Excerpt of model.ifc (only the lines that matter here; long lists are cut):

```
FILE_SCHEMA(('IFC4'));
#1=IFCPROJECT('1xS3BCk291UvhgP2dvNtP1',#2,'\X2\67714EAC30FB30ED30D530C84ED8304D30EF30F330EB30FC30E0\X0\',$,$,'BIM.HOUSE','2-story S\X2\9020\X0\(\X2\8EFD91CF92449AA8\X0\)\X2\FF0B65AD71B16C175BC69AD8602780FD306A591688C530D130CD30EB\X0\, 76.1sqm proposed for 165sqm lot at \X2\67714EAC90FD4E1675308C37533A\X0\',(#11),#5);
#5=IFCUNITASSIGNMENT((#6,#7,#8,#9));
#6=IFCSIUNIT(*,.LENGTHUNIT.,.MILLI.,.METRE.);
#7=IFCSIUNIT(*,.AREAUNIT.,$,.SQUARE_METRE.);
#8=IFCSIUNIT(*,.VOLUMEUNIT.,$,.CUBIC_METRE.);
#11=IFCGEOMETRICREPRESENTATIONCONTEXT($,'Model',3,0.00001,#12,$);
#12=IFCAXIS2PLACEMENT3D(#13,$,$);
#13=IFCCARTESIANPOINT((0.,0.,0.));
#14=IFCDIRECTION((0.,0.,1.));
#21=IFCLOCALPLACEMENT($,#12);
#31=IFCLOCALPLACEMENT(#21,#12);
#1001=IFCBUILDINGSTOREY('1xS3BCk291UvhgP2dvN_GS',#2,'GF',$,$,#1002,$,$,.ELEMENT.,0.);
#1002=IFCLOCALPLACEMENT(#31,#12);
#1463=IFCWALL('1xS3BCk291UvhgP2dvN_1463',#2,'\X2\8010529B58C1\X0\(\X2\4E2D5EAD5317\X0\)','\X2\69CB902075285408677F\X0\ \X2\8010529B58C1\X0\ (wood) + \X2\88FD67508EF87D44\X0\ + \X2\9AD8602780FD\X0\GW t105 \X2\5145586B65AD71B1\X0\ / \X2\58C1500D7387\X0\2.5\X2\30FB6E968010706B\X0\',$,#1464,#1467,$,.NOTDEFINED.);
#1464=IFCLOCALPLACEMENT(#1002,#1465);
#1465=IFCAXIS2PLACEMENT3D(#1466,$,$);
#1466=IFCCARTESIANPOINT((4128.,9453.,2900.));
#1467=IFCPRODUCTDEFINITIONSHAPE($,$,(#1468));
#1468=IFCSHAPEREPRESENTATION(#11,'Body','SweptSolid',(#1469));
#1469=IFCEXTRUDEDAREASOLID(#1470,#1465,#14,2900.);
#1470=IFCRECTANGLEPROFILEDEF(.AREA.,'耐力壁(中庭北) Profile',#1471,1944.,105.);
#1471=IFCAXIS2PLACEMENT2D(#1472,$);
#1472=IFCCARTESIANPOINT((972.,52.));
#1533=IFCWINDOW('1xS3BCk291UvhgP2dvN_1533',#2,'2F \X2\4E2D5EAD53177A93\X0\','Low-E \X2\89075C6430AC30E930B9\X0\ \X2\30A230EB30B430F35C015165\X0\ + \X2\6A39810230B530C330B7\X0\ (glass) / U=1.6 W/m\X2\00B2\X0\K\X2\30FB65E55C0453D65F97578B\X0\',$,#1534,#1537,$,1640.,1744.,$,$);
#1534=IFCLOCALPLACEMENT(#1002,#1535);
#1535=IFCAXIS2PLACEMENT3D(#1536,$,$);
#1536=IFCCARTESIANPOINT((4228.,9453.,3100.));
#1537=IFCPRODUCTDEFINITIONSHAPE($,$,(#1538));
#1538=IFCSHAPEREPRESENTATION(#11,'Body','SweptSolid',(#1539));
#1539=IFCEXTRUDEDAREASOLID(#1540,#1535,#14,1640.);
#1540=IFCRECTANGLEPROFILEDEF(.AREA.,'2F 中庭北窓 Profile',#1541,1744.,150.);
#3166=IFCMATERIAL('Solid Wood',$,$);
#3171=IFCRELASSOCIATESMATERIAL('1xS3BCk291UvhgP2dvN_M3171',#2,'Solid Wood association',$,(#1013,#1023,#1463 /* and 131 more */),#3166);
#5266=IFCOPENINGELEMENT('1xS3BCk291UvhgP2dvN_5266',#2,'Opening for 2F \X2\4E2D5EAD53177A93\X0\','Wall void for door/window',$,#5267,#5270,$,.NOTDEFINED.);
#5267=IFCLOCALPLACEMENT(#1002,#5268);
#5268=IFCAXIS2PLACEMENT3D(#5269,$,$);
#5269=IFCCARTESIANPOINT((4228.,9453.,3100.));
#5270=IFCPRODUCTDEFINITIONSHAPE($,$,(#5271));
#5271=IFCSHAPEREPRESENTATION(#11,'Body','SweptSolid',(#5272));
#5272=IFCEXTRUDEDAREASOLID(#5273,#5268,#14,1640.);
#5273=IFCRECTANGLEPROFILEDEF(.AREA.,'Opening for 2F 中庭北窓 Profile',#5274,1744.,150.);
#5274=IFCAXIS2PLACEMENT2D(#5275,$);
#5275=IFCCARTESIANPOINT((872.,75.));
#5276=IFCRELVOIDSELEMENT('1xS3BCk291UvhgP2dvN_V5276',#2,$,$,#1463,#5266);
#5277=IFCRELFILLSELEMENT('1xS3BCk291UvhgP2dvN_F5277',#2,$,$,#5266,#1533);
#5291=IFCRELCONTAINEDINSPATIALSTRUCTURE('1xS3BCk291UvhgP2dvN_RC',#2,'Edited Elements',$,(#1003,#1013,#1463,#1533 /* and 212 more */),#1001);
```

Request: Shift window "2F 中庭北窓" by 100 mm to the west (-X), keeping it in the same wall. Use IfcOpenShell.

```python
import ifcopenshell
import ifcopenshell.api.geometry
import ifcopenshell.util.placement

model = ifcopenshell.open("model.ifc")

window = model.by_guid("1xS3BCk291UvhgP2dvN_1533")
opening = window.FillsVoids[0].RelatingOpeningElement
wall = opening.VoidsElements[0].RelatingBuildingElement

wall_matrix = ifcopenshell.util.placement.get_local_placement(wall.ObjectPlacement)
shift = wall_matrix[:3, 0] * -100.0
before = ifcopenshell.util.placement.get_local_placement(window.ObjectPlacement)[:3, 3].copy()

# The window is not placed relative to its opening, so move both.
for product in (opening, window):
    matrix = ifcopenshell.util.placement.get_local_placement(product.ObjectPlacement)
    matrix[:3, 3] += shift
    ifcopenshell.api.geometry.edit_object_placement(model, product=product, matrix=matrix, is_si=False)

after = ifcopenshell.util.placement.get_local_placement(window.ObjectPlacement)[:3, 3]
print("window moved by", (after - before).round(3) + 0.0)

model.write("model_updated.ifc")
```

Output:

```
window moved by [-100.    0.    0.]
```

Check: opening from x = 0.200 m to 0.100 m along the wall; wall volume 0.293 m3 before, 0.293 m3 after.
